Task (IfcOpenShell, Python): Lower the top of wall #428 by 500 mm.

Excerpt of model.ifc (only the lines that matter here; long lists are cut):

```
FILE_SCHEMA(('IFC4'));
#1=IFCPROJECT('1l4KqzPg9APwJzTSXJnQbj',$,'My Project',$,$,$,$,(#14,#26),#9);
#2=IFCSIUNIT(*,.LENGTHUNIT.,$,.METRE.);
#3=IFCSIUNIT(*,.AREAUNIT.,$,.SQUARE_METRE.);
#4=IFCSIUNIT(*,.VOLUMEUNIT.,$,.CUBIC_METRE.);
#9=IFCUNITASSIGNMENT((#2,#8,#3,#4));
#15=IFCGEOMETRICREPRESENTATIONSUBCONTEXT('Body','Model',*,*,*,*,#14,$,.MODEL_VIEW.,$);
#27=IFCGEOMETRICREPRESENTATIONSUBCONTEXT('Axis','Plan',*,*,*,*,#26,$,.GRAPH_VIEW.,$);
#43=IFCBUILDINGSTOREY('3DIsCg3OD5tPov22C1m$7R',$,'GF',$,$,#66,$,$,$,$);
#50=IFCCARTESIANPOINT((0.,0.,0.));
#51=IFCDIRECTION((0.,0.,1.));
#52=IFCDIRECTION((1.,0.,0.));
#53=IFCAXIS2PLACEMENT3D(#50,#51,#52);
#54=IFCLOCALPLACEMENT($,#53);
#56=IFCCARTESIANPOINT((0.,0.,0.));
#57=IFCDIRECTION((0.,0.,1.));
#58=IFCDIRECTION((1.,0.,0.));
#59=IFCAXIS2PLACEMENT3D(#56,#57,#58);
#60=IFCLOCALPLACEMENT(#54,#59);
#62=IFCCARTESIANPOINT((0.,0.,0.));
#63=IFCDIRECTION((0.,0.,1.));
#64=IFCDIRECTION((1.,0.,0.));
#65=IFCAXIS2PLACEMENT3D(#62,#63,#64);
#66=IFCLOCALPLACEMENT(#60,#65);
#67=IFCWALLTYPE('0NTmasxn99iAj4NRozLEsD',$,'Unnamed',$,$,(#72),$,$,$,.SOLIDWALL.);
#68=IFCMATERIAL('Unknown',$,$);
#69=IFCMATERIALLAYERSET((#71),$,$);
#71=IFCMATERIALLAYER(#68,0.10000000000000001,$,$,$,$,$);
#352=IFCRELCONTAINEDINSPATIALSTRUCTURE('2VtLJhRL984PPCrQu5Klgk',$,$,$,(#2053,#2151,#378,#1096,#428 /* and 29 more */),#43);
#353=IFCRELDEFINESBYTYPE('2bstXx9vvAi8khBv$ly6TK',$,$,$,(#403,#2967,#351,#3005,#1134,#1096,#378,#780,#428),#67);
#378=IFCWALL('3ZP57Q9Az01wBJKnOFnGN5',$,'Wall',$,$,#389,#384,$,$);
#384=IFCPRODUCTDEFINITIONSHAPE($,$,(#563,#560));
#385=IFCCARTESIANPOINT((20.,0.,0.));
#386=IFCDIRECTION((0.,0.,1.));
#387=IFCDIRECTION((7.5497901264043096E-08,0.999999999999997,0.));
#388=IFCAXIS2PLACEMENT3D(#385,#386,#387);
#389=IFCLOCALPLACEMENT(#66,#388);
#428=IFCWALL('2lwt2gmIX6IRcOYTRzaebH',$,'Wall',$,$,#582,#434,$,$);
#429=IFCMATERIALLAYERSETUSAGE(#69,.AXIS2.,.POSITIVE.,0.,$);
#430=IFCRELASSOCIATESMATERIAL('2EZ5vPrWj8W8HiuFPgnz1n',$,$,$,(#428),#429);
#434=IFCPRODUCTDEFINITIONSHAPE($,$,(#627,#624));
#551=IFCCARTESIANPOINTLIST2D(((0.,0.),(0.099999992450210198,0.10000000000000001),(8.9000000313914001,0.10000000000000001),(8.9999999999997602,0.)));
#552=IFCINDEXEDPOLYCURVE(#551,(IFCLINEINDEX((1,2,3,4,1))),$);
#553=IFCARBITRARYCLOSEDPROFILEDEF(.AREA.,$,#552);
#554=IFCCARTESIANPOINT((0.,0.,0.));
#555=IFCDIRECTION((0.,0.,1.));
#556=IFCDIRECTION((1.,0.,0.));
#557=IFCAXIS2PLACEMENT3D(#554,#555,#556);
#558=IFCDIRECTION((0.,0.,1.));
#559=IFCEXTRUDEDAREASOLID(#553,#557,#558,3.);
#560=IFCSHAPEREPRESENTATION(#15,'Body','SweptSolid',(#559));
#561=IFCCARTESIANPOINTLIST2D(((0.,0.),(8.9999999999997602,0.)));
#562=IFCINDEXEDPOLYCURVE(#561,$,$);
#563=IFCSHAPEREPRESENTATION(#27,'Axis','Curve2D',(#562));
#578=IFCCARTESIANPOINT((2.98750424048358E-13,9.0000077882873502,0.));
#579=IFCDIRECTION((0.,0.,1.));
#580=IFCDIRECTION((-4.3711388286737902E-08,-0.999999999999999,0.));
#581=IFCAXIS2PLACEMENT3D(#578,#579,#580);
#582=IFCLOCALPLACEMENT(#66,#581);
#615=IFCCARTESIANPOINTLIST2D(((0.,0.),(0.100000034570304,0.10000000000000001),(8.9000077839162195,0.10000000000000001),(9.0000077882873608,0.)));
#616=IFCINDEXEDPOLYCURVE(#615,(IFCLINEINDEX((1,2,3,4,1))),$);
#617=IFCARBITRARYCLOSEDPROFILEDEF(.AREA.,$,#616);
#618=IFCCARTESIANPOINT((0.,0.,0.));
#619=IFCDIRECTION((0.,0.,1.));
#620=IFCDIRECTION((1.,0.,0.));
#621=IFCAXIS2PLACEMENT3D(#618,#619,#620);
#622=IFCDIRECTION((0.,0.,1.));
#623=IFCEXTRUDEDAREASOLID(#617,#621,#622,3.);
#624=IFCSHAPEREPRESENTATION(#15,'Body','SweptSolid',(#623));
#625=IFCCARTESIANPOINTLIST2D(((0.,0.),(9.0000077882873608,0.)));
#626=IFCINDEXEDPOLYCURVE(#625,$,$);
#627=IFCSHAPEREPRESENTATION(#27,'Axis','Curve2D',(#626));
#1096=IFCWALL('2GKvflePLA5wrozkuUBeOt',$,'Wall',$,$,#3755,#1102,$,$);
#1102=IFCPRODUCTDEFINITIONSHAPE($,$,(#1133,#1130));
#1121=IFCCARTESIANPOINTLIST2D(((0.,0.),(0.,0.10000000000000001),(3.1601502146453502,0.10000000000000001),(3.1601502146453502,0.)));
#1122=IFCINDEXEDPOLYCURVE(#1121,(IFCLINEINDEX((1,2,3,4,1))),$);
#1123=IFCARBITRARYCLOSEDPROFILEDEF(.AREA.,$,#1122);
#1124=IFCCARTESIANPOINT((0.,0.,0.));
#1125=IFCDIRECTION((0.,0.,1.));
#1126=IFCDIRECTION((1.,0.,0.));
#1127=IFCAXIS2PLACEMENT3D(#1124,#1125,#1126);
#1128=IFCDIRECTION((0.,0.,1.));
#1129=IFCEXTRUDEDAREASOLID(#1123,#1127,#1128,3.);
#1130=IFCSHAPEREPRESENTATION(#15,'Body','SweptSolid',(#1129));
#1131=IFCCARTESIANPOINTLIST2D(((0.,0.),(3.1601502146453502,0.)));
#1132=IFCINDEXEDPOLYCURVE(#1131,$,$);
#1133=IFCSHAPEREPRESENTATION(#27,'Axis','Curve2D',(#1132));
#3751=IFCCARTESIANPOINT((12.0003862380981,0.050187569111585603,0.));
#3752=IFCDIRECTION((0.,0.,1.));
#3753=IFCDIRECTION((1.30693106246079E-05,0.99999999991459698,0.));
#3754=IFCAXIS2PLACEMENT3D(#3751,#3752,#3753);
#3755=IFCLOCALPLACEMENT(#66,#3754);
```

```python
import ifcopenshell
import ifcopenshell.geom
import ifcopenshell.util.representation
import ifcopenshell.util.shape
import ifcopenshell.util.unit

model = ifcopenshell.open("model.ifc")
unit_scale = ifcopenshell.util.unit.calculate_unit_scale(model)
settings = ifcopenshell.geom.settings()


def volume(element):
    """Net volume in cubic metres, openings subtracted."""
    shape = ifcopenshell.geom.create_shape(settings, element)
    return ifcopenshell.util.shape.get_volume(shape.geometry)


wall = model.by_guid("2lwt2gmIX6IRcOYTRzaebH")
before = volume(wall)

body = ifcopenshell.util.representation.get_representation(wall, "Model", "Body")
solid = body.Items[0]
old_height = solid.Depth
solid.Depth -= 0.5 / unit_scale
after = volume(wall)

print(f"height {old_height:g} -> {solid.Depth:g}, volume {before:.3f} -> {after:.3f} m3")

model.write("model-out.ifc")
```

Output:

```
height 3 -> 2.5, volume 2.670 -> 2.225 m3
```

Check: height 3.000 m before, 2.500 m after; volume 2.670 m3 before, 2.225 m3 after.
